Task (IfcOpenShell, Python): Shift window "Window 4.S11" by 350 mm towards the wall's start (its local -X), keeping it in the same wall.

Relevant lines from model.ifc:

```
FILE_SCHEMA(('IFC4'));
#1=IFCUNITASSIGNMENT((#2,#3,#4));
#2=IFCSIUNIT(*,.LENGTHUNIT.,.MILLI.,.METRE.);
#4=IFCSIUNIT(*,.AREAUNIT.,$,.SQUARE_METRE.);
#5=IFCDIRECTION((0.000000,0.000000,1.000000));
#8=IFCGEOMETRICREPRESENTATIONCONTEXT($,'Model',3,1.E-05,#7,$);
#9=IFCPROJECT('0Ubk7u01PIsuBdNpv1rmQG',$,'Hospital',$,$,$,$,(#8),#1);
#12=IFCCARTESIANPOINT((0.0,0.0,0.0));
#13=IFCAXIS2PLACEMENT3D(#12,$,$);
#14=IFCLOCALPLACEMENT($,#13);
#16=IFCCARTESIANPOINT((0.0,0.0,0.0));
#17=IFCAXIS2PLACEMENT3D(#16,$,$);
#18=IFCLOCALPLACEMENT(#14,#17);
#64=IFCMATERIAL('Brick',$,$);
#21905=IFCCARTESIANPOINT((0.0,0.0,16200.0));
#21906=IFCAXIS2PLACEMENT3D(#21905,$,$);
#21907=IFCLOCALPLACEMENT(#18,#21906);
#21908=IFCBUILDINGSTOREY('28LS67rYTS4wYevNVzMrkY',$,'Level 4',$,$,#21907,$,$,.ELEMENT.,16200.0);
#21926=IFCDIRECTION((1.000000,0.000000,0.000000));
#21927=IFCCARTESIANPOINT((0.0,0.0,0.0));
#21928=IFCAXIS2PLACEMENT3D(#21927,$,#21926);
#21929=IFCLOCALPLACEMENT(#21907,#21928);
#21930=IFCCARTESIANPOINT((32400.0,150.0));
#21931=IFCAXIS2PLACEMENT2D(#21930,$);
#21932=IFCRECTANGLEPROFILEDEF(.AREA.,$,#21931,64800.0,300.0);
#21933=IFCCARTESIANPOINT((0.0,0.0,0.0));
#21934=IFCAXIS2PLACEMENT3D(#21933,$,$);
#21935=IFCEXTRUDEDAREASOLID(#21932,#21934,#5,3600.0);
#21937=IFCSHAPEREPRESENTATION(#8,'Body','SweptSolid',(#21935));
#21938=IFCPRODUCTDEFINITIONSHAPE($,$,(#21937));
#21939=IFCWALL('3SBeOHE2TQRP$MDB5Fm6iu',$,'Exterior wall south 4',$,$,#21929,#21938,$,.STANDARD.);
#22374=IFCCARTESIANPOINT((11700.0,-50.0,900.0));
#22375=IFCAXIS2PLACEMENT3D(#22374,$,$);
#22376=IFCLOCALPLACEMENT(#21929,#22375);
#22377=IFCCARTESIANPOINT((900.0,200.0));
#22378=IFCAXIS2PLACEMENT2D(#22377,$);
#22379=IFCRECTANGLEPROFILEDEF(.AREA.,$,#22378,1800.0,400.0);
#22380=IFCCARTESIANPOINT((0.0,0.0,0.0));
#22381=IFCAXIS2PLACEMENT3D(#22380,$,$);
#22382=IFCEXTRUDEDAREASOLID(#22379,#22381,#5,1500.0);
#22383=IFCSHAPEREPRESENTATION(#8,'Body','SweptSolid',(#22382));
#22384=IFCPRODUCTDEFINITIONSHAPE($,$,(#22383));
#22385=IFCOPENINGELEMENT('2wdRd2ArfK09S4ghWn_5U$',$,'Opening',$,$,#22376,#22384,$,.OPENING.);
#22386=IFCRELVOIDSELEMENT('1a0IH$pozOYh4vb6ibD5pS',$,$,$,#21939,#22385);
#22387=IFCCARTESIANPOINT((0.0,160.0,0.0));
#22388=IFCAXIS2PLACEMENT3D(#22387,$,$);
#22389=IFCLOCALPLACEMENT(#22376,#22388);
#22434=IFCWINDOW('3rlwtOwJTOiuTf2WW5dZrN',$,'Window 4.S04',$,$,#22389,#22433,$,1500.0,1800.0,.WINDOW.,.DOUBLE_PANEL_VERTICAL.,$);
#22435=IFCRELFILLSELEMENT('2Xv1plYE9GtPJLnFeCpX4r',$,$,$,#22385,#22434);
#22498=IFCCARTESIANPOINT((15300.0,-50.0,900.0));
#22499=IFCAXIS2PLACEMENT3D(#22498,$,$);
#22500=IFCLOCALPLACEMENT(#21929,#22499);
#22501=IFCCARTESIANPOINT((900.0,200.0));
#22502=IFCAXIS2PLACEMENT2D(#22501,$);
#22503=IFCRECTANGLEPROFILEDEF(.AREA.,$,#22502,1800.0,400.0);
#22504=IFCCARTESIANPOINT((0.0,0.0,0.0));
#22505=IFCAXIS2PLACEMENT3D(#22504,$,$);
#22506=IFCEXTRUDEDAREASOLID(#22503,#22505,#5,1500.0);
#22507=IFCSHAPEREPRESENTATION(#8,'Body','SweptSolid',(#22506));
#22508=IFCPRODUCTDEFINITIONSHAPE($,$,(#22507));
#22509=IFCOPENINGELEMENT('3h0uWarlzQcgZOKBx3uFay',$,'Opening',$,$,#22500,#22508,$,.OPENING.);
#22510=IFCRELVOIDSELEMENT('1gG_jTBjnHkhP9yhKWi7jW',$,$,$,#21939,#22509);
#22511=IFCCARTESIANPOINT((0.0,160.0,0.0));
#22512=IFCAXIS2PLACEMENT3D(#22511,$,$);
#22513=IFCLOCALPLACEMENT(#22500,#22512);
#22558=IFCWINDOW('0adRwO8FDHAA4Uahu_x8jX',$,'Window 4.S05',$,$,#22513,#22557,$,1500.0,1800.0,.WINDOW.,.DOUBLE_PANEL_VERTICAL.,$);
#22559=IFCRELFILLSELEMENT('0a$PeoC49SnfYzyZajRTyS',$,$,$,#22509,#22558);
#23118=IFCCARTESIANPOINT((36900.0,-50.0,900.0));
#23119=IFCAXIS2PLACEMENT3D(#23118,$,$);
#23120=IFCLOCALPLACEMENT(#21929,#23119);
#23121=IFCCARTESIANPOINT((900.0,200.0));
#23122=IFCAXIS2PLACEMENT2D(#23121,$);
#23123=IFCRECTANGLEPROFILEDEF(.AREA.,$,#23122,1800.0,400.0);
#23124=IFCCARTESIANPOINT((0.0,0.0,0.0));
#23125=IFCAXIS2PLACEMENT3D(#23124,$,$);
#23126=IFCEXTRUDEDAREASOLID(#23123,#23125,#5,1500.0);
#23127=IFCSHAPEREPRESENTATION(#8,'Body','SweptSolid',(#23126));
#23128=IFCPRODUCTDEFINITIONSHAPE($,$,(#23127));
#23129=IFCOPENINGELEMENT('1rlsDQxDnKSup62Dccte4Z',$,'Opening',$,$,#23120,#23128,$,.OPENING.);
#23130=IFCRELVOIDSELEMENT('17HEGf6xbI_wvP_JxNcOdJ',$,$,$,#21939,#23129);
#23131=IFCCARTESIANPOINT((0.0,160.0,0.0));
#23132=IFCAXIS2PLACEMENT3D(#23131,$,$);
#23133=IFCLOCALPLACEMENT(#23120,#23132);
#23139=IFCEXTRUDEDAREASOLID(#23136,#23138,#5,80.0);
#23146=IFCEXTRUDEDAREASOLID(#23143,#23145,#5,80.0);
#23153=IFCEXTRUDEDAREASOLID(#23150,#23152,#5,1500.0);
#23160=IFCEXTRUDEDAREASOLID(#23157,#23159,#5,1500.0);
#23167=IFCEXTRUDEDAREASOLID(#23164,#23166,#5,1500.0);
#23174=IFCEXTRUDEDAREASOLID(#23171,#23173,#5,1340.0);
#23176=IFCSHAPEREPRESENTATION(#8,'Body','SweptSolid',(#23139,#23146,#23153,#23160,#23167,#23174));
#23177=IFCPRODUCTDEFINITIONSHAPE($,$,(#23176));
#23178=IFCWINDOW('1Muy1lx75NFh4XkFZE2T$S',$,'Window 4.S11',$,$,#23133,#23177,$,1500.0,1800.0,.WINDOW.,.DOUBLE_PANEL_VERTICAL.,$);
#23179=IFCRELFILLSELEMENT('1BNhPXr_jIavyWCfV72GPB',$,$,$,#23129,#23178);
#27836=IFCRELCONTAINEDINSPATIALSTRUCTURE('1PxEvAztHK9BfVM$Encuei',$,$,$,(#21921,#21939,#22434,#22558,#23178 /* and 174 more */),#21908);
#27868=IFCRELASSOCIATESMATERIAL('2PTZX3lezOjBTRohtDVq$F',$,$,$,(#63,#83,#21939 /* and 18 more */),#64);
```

```python
import ifcopenshell
import ifcopenshell.api.geometry
import ifcopenshell.util.placement
import ifcopenshell.util.unit

model = ifcopenshell.open("model.ifc")
unit_scale = ifcopenshell.util.unit.calculate_unit_scale(model)

window = model.by_guid("1Muy1lx75NFh4XkFZE2T$S")
opening = window.FillsVoids[0].RelatingOpeningElement
wall = opening.VoidsElements[0].RelatingBuildingElement

wall_matrix = ifcopenshell.util.placement.get_local_placement(wall.ObjectPlacement)
shift = wall_matrix[:3, 0] * -0.35 / unit_scale
before = ifcopenshell.util.placement.get_local_placement(window.ObjectPlacement)[:3, 3].copy()

# The window is placed relative to its opening, so it follows when the opening moves.
matrix = ifcopenshell.util.placement.get_local_placement(opening.ObjectPlacement)
matrix[:3, 3] += shift
ifcopenshell.api.geometry.edit_object_placement(
    model, product=opening, matrix=matrix, is_si=False, should_transform_children=True
)

after = ifcopenshell.util.placement.get_local_placement(window.ObjectPlacement)[:3, 3]
print("window moved by", (after - before).round(3) + 0.0)

model.write("model_updated.ifc")
```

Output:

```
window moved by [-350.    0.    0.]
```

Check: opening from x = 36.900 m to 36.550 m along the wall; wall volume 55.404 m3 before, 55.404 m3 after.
